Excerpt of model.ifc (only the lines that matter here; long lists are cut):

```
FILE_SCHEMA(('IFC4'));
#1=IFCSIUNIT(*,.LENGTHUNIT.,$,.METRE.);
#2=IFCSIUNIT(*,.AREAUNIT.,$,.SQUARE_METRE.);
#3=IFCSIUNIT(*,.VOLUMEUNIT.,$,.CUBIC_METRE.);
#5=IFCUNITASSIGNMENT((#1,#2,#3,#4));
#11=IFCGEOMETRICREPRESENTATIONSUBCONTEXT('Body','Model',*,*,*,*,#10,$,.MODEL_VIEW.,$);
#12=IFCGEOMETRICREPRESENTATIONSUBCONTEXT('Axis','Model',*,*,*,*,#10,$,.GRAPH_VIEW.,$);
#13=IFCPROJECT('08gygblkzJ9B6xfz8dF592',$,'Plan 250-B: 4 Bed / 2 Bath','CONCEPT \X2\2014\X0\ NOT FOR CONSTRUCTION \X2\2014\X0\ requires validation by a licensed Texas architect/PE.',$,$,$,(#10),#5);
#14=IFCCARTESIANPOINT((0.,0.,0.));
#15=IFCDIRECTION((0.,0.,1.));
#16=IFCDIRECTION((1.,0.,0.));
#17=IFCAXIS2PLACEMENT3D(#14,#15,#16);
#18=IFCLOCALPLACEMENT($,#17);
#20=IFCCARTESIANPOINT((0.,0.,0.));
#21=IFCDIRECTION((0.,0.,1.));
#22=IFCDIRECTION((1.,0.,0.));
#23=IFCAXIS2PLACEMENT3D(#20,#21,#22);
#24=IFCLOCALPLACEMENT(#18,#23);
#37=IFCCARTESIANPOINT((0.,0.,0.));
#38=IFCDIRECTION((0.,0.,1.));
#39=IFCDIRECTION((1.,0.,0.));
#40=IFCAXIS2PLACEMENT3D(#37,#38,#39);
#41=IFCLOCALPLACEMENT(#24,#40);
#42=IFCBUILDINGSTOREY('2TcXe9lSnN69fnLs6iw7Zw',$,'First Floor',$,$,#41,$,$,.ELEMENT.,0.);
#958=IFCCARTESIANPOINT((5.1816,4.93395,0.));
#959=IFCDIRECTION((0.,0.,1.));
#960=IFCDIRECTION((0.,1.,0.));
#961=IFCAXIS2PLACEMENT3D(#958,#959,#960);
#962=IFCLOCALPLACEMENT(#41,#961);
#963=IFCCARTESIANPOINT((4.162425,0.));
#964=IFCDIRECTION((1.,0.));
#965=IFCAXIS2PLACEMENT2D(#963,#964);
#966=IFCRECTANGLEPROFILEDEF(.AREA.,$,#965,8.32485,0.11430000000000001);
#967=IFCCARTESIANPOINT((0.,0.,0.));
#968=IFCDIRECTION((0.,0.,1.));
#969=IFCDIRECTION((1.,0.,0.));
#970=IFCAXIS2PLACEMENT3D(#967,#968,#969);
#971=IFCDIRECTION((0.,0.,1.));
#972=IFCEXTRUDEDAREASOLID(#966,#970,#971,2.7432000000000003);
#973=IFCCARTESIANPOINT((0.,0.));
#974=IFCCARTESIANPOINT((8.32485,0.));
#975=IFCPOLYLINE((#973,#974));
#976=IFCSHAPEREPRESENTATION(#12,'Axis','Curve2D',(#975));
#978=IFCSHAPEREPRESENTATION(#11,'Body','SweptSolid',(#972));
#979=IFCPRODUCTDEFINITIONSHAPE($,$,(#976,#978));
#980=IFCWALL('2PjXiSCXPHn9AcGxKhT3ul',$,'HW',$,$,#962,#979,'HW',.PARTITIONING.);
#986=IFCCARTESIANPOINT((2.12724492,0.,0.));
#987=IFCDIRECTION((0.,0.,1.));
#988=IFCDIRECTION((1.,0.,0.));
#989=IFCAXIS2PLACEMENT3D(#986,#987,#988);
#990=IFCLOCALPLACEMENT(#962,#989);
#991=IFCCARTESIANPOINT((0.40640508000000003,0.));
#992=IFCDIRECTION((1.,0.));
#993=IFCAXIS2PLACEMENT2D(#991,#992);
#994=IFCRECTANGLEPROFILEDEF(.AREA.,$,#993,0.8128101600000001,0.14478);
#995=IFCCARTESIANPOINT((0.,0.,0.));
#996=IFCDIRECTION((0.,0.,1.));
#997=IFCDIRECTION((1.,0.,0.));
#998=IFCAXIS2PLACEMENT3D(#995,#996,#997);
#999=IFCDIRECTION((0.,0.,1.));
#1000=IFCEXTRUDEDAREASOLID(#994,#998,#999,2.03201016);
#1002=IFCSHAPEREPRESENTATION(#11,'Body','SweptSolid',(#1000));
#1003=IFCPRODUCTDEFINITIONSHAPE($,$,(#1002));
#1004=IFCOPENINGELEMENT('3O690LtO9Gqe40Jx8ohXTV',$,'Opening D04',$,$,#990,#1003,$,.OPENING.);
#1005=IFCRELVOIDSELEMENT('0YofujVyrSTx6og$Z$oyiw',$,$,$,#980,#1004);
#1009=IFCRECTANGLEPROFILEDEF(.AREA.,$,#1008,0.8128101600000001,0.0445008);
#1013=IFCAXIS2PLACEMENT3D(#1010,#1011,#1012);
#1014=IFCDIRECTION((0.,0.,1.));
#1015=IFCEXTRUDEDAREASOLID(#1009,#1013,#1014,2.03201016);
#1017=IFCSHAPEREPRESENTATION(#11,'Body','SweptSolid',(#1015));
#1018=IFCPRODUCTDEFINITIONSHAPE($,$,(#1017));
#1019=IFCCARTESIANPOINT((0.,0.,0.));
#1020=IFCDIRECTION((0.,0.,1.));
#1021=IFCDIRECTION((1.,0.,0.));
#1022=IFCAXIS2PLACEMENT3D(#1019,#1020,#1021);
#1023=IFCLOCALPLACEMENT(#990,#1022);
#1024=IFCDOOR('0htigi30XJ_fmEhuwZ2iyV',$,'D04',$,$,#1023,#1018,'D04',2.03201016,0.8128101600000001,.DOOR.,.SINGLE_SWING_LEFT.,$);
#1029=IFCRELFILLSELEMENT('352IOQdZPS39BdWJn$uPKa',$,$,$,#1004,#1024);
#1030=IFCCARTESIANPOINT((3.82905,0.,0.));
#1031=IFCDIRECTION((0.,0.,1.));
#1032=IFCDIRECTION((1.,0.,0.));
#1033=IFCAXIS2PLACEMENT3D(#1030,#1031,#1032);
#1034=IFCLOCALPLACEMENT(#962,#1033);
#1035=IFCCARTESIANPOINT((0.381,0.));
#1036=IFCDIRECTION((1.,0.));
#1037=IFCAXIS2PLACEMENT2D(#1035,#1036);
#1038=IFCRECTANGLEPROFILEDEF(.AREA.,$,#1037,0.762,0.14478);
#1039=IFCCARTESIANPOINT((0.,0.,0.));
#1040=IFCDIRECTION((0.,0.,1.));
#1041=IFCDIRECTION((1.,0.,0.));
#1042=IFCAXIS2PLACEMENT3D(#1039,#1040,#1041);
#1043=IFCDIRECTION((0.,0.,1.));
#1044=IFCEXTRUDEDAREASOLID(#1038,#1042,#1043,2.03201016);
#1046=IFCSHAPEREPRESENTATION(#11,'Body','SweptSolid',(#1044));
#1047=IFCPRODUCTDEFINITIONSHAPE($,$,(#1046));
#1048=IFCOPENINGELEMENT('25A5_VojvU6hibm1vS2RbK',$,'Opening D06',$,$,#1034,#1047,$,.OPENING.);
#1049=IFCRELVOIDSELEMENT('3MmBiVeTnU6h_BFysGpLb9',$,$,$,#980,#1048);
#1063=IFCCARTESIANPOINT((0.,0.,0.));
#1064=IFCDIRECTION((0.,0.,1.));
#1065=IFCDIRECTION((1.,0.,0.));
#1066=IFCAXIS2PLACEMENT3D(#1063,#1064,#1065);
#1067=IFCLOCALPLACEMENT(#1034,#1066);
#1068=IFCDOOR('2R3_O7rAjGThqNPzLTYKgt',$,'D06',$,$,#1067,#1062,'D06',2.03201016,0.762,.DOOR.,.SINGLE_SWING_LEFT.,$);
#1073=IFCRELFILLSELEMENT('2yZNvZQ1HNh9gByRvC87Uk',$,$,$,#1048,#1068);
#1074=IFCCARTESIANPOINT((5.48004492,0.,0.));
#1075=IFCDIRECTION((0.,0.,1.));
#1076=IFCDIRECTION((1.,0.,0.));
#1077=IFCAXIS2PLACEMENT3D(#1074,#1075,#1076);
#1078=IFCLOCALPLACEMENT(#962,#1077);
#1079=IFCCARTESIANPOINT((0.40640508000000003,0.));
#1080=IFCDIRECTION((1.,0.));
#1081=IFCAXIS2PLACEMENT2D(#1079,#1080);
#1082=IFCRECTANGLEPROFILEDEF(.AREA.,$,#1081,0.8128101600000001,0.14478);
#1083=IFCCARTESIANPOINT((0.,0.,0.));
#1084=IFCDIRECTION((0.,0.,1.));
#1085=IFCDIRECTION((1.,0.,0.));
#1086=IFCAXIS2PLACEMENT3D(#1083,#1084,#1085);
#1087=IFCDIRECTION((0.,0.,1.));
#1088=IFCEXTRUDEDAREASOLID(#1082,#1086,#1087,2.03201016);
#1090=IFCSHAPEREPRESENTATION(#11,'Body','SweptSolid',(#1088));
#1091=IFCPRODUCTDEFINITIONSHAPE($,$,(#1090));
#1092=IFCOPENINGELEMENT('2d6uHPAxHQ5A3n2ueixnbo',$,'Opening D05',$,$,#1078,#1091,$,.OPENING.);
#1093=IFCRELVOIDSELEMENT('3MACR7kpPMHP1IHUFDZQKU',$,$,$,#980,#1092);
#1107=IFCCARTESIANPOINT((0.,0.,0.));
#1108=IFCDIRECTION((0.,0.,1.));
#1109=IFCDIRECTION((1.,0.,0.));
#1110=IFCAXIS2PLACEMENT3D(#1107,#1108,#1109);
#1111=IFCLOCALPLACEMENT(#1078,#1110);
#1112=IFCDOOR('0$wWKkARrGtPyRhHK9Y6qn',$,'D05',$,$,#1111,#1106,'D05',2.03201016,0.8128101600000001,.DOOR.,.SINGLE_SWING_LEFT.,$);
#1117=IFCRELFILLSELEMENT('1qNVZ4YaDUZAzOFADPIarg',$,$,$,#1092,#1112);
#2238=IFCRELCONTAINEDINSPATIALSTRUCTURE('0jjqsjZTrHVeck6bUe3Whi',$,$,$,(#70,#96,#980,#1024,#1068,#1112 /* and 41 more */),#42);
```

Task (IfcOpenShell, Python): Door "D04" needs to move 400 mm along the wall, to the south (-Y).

```python
import ifcopenshell
import ifcopenshell.api.geometry
import ifcopenshell.util.placement
import ifcopenshell.util.unit

model = ifcopenshell.open("model.ifc")
unit_scale = ifcopenshell.util.unit.calculate_unit_scale(model)

door = model.by_id(1024)
opening = door.FillsVoids[0].RelatingOpeningElement
wall = opening.VoidsElements[0].RelatingBuildingElement

wall_matrix = ifcopenshell.util.placement.get_local_placement(wall.ObjectPlacement)
shift = wall_matrix[:3, 0] * -0.4 / unit_scale
before = ifcopenshell.util.placement.get_local_placement(door.ObjectPlacement)[:3, 3].copy()

# The door is placed relative to its opening, so it follows when the opening moves.
matrix = ifcopenshell.util.placement.get_local_placement(opening.ObjectPlacement)
matrix[:3, 3] += shift
ifcopenshell.api.geometry.edit_object_placement(
    model, product=opening, matrix=matrix, is_si=False, should_transform_children=True
)

after = ifcopenshell.util.placement.get_local_placement(door.ObjectPlacement)[:3, 3]
print("door moved by", (after - before).round(3) + 0.0)

model.write("model_updated.ifc")
```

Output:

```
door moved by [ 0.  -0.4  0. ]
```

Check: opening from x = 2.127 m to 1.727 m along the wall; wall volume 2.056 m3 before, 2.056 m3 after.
